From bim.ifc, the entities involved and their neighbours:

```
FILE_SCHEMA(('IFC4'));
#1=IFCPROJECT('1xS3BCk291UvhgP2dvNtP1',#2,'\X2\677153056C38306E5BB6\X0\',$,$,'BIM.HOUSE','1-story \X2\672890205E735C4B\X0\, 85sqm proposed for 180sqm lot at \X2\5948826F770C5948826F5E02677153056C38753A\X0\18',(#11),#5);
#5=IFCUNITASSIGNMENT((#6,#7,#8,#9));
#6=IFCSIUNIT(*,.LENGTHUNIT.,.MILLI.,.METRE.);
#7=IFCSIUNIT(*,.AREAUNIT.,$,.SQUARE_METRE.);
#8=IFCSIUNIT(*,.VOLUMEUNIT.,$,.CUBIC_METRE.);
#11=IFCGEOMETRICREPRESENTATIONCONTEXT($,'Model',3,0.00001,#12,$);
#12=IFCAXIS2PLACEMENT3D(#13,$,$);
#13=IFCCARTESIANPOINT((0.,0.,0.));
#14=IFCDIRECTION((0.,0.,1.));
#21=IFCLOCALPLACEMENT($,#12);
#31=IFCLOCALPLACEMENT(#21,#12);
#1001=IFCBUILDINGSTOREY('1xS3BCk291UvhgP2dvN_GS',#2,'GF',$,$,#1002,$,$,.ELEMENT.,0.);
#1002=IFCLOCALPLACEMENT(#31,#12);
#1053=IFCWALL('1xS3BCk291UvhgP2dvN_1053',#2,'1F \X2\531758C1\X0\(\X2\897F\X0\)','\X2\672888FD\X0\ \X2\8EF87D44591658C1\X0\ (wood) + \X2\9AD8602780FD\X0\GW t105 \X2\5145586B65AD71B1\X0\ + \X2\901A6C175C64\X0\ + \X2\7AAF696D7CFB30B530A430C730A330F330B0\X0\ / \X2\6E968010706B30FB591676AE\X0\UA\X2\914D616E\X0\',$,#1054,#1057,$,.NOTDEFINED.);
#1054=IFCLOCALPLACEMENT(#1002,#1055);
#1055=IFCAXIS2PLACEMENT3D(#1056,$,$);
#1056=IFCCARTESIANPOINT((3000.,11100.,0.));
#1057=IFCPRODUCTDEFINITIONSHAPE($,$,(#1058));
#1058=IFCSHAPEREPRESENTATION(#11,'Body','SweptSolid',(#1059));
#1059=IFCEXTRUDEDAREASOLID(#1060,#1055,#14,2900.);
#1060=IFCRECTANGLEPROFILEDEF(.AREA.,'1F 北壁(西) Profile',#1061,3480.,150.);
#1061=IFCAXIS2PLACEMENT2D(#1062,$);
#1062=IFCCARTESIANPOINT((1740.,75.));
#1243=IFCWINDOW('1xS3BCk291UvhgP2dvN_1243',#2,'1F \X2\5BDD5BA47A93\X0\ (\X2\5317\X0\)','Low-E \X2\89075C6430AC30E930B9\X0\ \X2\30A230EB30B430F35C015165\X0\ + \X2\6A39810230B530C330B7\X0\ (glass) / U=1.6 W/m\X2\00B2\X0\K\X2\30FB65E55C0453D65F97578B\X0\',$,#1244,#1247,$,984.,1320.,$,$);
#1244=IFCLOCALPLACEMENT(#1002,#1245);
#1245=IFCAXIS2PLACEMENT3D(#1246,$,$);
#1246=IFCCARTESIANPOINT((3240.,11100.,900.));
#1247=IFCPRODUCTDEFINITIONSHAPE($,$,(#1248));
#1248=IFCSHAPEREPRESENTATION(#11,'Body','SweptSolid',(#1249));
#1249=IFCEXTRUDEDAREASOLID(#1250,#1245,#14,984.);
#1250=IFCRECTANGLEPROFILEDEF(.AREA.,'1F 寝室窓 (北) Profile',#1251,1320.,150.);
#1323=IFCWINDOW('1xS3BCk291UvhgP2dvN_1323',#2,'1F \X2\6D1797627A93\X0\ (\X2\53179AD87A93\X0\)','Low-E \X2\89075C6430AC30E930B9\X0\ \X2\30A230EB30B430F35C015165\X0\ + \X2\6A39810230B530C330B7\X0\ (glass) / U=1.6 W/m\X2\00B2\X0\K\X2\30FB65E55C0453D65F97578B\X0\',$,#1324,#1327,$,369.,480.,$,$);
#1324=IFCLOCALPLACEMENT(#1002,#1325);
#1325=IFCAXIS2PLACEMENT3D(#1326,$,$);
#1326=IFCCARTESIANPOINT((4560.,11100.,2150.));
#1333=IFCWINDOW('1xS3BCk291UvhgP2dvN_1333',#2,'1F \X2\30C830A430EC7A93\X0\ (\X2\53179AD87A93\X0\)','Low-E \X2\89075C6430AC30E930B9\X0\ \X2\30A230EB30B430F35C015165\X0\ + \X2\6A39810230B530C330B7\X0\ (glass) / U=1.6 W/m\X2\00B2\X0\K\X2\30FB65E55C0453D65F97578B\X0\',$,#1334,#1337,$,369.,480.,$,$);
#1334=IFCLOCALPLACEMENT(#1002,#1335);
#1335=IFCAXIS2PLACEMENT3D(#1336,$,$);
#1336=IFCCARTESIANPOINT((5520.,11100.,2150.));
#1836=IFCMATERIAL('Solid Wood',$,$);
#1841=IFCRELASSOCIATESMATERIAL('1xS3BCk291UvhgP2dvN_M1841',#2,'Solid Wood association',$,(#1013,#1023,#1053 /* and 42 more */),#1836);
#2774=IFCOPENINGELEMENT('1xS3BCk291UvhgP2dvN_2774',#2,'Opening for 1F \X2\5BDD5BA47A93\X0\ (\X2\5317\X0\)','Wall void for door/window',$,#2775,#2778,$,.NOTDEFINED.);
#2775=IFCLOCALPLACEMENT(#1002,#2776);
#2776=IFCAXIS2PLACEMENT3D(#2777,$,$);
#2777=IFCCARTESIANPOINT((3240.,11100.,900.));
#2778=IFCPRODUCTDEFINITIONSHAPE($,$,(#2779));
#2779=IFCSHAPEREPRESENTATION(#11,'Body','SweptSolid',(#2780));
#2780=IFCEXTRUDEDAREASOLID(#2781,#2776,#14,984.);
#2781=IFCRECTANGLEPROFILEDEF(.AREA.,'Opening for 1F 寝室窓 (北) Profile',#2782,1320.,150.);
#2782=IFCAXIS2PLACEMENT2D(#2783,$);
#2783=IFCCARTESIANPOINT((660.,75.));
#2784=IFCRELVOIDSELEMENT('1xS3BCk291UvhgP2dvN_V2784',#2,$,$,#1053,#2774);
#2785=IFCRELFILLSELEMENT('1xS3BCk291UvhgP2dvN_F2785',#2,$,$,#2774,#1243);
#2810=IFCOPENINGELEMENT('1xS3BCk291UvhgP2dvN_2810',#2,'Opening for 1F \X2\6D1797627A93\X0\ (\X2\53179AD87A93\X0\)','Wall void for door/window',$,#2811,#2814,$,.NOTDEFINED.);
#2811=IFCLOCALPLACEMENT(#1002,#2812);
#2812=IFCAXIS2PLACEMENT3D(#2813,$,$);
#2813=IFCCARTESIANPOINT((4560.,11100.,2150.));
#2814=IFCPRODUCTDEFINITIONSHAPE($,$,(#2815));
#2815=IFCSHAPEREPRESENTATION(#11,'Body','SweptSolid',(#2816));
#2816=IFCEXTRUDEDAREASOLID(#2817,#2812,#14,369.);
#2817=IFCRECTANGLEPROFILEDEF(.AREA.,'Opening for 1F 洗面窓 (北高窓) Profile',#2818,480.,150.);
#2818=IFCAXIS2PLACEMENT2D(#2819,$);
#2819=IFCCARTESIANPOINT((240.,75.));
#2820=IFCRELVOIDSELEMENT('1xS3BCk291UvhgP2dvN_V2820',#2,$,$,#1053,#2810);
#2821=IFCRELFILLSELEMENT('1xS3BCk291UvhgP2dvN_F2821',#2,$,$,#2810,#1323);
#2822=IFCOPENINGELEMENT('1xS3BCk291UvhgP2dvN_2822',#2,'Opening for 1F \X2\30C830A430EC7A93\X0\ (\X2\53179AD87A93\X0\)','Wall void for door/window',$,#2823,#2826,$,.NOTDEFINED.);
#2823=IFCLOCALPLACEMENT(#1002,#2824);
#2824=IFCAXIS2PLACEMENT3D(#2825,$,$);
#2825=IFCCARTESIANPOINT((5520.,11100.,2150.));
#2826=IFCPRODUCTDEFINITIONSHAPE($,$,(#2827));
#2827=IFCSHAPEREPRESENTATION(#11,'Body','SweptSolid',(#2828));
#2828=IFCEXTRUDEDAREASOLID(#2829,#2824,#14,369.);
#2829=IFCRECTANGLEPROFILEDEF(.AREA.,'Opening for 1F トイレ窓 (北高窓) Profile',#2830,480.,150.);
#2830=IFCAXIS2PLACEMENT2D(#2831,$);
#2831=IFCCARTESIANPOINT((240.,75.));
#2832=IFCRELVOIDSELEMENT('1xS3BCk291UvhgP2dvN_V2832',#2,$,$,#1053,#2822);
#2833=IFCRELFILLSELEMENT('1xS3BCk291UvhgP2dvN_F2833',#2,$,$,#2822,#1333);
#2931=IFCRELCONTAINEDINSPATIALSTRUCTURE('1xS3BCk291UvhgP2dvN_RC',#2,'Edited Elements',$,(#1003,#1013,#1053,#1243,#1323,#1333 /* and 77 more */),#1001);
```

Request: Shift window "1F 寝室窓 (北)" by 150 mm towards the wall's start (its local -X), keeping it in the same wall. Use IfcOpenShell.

```python
import ifcopenshell
import ifcopenshell.api.geometry
import ifcopenshell.util.placement
import ifcopenshell.util.unit

model = ifcopenshell.open("bim.ifc")
unit_scale = ifcopenshell.util.unit.calculate_unit_scale(model)

window = model.by_id(1243)
opening = window.FillsVoids[0].RelatingOpeningElement
wall = opening.VoidsElements[0].RelatingBuildingElement

wall_matrix = ifcopenshell.util.placement.get_local_placement(wall.ObjectPlacement)
shift = wall_matrix[:3, 0] * -0.15 / unit_scale
before = ifcopenshell.util.placement.get_local_placement(window.ObjectPlacement)[:3, 3].copy()

# The window is not placed relative to its opening, so move both.
for product in (opening, window):
    matrix = ifcopenshell.util.placement.get_local_placement(product.ObjectPlacement)
    matrix[:3, 3] += shift
    ifcopenshell.api.geometry.edit_object_placement(model, product=product, matrix=matrix, is_si=False)

after = ifcopenshell.util.placement.get_local_placement(window.ObjectPlacement)[:3, 3]
print("window moved by", (after - before).round(3) + 0.0)

model.write("bim_updated.ifc")
```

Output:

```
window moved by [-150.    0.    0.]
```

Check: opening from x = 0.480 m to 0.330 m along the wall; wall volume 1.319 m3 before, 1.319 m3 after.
